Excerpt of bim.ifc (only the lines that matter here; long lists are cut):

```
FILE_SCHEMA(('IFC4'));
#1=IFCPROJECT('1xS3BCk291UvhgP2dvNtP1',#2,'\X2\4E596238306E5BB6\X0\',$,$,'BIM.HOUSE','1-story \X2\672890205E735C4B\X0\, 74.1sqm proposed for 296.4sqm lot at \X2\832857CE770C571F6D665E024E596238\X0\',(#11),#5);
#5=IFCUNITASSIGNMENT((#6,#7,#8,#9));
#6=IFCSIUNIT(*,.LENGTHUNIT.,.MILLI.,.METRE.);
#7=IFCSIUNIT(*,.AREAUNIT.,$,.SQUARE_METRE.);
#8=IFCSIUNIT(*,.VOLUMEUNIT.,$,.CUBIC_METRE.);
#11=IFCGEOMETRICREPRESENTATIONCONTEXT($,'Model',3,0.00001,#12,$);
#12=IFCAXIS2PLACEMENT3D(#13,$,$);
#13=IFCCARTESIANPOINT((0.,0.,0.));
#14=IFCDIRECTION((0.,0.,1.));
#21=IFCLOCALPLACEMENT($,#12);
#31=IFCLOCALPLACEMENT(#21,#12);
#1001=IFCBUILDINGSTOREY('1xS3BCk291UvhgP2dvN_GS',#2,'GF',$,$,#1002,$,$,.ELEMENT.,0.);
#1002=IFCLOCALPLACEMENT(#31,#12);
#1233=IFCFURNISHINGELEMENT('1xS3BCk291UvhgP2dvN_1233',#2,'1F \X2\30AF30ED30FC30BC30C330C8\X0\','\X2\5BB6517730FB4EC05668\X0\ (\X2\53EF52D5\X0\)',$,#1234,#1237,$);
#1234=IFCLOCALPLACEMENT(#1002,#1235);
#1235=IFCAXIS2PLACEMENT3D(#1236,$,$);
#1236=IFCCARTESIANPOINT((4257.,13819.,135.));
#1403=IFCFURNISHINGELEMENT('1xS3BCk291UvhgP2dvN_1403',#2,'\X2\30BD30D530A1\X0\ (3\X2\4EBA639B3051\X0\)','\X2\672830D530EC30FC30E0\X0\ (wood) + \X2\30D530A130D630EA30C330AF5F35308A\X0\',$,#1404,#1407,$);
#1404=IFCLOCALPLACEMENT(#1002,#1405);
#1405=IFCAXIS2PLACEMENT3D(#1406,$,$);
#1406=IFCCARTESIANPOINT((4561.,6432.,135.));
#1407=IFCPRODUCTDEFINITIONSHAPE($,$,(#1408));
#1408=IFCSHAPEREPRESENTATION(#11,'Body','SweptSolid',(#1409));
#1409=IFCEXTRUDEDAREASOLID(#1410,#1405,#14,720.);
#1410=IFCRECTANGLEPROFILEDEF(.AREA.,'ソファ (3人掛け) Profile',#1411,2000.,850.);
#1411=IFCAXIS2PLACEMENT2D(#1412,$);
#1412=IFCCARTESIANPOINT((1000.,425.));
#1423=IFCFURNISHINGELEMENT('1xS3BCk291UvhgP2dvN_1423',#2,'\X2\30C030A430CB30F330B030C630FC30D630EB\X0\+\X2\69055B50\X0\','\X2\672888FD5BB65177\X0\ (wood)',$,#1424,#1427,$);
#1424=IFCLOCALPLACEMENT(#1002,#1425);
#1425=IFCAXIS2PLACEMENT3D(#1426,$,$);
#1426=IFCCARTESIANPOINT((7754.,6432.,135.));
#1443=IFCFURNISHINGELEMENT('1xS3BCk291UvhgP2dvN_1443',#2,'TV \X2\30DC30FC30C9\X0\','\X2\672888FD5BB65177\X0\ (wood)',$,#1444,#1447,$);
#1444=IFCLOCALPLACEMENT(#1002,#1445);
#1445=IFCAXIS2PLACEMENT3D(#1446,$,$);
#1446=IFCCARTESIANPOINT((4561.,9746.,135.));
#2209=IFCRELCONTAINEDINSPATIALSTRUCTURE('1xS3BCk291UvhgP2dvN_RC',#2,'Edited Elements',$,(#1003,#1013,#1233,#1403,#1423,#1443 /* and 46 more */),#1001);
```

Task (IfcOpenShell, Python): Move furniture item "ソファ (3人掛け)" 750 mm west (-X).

```python
import ifcopenshell
import ifcopenshell.api.geometry
import ifcopenshell.util.placement

model = ifcopenshell.open("bim.ifc")

item = model.by_guid("1xS3BCk291UvhgP2dvN_1403")
matrix = ifcopenshell.util.placement.get_local_placement(item.ObjectPlacement)
matrix[0, 3] -= 750.0
ifcopenshell.api.geometry.edit_object_placement(model, product=item, matrix=matrix, is_si=False)

print(ifcopenshell.util.placement.get_local_placement(item.ObjectPlacement).round(3) + 0.0)

model.write("bim_edited.ifc")
```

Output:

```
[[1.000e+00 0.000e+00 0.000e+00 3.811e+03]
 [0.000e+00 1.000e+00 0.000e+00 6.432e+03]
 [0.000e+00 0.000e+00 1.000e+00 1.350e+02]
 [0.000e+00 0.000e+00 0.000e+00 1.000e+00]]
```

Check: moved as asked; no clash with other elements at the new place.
